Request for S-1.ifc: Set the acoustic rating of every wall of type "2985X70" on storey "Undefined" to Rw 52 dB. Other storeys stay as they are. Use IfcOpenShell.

First a look at what the model holds.

```python
import ifcopenshell
import ifcopenshell.util.element

model = ifcopenshell.open("S-1.ifc")
print(model.schema)
storey = next(s for s in model.by_type("IfcBuildingStorey") if s.Name == "Undefined")
walls = [e for e in ifcopenshell.util.element.get_decomposition(storey) if e.is_a("IfcWall")]
seen = {}
for e in walls:
    element_type = ifcopenshell.util.element.get_type(e)
    key = (element_type.Name if element_type != e and element_type else None, ifcopenshell.util.element.get_pset(e, "Pset_WallCommon", "AcousticRating"))
    seen[key] = seen.get(key, 0) + 1
for (name, value), count in sorted(seen.items(), key=str):
    print(count, "x", name, "|", value)
```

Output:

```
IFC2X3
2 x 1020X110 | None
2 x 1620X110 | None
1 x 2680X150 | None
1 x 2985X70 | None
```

```python
import ifcopenshell
import ifcopenshell.api.pset
import ifcopenshell.util.element

model = ifcopenshell.open("S-1.ifc")

storey = next(s for s in model.by_type("IfcBuildingStorey") if s.Name == "Undefined")
walls = [e for e in ifcopenshell.util.element.get_decomposition(storey) if e.is_a("IfcWall")]

count = 0
for e in walls:
    element_type = ifcopenshell.util.element.get_type(e)
    if element_type in (None, e) or element_type.Name != "2985X70":
        continue
    # add_pset returns the element's existing set when there is one.
    pset = ifcopenshell.api.pset.add_pset(model, product=e, name="Pset_WallCommon")
    ifcopenshell.api.pset.edit_pset(model, pset=pset, properties={"AcousticRating": "Rw 52 dB"})
    count += 1

print(count, "walls updated")

model.write("S-1_v2.ifc")
```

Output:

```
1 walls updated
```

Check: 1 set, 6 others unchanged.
